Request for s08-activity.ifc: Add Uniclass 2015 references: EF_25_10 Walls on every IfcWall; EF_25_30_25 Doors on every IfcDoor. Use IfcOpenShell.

First a look at what the model holds.

```python
import ifcopenshell

model = ifcopenshell.open("s08-activity.ifc")
print(model.schema)
print("classifications:", [c.Name for c in model.by_type("IfcClassification")])
for ifc_class in ("IfcDoor", "IfcRoof", "IfcStair", "IfcWall", "IfcWindow"):
    print(ifc_class, len(model.by_type(ifc_class)))
```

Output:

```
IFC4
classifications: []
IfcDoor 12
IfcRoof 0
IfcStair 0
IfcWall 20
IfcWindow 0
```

```python
import ifcopenshell
import ifcopenshell.api.classification

model = ifcopenshell.open("s08-activity.ifc")

system = ifcopenshell.api.classification.add_classification(model, classification="Uniclass 2015")

codes = {
    "IfcWall": ("EF_25_10", "Walls"),
    "IfcDoor": ("EF_25_30_25", "Doors"),
}
for ifc_class, (code, name) in codes.items():
    products = model.by_type(ifc_class)
    ifcopenshell.api.classification.add_reference(
        model, products=products, classification=system, identification=code, name=name
    )
    print(code, len(products))

model.write("s08-activity_v2.ifc")
```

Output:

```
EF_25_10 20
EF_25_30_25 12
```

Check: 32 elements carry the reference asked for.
